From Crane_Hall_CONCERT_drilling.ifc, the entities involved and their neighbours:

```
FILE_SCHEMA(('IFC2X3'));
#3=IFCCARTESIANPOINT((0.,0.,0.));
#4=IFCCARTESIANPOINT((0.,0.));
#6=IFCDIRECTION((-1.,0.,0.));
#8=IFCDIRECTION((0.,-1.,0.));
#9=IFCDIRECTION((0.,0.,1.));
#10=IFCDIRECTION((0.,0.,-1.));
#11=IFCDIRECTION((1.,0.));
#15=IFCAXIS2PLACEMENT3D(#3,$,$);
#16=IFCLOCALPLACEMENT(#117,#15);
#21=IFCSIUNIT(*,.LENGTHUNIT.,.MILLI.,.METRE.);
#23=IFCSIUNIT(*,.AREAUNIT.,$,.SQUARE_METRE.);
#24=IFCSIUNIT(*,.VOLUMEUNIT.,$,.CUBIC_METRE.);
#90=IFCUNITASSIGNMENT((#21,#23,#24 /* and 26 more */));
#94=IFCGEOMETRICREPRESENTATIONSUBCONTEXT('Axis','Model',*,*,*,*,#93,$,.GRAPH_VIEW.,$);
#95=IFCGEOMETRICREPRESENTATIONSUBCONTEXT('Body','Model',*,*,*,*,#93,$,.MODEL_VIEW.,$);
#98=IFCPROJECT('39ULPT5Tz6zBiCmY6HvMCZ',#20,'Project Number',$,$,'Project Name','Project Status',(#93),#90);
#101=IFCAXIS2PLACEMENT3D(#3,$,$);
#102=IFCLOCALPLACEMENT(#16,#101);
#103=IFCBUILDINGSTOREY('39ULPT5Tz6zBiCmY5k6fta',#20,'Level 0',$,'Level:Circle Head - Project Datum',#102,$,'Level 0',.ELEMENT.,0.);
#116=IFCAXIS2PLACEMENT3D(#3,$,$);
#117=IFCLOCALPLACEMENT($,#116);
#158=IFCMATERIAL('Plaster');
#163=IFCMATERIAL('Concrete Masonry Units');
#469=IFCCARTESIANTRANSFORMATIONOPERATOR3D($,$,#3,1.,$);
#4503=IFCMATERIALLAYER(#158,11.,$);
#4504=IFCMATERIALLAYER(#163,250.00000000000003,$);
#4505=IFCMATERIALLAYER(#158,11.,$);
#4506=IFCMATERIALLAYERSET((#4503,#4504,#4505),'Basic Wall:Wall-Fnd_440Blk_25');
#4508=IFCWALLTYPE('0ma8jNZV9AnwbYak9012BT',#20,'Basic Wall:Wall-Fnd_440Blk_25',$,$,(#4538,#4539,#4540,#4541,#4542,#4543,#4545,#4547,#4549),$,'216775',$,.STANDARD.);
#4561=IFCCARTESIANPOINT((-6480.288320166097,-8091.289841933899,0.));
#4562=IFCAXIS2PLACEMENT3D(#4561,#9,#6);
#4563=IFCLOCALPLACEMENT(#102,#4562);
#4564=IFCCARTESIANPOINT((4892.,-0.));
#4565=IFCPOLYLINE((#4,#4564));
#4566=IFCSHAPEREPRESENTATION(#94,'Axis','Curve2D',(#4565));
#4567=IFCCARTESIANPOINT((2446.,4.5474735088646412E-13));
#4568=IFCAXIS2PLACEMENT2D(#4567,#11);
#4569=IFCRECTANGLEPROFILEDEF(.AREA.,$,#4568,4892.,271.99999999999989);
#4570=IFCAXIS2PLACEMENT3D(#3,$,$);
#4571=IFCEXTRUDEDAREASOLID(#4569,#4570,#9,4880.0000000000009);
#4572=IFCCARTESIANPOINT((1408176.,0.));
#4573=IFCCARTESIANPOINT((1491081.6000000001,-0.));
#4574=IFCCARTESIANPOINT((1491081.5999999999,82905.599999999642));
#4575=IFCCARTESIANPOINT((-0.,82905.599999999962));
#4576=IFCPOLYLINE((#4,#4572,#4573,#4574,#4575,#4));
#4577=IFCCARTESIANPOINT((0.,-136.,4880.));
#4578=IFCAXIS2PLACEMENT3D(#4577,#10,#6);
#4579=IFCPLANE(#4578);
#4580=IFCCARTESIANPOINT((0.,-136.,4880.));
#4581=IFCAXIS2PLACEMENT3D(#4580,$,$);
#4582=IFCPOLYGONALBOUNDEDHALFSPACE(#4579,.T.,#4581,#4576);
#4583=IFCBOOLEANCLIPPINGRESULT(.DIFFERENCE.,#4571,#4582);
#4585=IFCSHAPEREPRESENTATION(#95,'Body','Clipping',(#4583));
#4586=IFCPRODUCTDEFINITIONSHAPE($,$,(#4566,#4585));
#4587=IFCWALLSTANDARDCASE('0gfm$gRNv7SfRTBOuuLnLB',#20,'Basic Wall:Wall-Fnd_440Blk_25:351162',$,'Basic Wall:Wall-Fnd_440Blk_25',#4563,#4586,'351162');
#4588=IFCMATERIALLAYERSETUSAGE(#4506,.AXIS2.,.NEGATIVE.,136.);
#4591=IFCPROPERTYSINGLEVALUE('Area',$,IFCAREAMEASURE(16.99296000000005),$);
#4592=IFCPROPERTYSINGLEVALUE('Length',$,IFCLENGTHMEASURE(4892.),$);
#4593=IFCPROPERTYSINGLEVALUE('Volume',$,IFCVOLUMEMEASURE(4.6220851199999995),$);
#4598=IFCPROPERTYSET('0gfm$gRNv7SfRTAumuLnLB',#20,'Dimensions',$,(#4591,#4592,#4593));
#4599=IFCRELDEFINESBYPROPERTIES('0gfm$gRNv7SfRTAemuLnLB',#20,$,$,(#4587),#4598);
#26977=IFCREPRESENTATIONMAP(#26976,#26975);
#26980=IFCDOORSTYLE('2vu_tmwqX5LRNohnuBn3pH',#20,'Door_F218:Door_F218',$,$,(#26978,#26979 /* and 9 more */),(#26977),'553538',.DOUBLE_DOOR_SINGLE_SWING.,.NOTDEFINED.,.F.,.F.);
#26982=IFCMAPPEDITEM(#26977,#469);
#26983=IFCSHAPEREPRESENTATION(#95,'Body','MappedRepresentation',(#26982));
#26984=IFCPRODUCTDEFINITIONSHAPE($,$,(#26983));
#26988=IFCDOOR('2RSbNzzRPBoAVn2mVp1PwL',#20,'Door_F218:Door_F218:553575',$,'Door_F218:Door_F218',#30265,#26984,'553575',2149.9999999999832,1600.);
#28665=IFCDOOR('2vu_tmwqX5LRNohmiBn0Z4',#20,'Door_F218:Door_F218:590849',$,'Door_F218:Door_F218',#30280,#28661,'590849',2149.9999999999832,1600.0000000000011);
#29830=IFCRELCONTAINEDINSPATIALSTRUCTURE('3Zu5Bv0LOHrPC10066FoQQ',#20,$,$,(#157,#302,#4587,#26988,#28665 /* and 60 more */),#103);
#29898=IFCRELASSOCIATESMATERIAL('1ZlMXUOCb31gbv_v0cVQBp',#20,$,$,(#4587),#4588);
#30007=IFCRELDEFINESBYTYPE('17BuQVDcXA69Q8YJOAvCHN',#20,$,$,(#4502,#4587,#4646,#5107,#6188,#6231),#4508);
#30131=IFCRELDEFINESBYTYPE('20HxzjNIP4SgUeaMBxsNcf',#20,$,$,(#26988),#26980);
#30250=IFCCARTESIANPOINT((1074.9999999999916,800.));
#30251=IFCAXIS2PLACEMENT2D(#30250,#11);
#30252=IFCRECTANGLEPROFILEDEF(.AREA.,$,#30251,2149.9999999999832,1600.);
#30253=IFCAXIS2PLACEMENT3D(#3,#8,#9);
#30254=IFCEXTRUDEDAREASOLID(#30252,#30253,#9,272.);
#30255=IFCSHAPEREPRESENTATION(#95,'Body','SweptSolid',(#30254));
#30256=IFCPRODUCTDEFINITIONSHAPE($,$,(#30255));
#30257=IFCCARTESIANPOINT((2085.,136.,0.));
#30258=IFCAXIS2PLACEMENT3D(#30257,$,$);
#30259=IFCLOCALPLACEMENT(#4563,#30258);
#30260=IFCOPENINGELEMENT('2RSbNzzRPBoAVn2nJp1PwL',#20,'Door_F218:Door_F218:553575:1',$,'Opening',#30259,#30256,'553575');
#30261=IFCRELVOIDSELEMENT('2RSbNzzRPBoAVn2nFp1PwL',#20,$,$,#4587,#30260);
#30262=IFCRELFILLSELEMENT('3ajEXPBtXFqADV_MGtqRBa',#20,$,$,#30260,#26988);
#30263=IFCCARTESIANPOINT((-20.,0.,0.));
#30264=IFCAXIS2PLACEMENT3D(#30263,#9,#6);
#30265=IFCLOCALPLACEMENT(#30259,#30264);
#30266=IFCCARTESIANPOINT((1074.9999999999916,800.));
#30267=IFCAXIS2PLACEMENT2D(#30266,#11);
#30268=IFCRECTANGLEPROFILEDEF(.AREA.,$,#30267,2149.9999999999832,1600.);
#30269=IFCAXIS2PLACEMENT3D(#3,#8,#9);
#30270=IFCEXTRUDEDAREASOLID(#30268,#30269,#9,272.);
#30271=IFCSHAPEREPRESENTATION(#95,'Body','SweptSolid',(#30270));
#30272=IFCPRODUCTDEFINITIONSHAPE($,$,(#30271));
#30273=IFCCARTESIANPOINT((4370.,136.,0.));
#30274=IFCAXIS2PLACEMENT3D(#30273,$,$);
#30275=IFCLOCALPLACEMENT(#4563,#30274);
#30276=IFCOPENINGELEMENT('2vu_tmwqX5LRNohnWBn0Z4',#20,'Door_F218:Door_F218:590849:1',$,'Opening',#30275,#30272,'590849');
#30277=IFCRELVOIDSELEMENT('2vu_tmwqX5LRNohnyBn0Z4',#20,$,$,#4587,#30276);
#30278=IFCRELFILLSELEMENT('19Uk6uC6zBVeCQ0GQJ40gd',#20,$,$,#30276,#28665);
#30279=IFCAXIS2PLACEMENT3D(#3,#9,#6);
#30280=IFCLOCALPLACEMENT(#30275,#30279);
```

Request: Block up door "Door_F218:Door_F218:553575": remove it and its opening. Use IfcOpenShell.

```python
import ifcopenshell
import ifcopenshell.api.feature
import ifcopenshell.api.pset
import ifcopenshell.api.root
import ifcopenshell.geom
import ifcopenshell.util.element
import ifcopenshell.util.shape
import ifcopenshell.util.unit

model = ifcopenshell.open("Crane_Hall_CONCERT_drilling.ifc")
area_scale = ifcopenshell.util.unit.calculate_unit_scale(model, "AREAUNIT")
volume_scale = ifcopenshell.util.unit.calculate_unit_scale(model, "VOLUMEUNIT")
settings = ifcopenshell.geom.settings()


def volume(element):
    """Net volume in cubic metres, openings subtracted."""
    shape = ifcopenshell.geom.create_shape(settings, element)
    return ifcopenshell.util.shape.get_volume(shape.geometry)


door = model.by_guid("2RSbNzzRPBoAVn2mVp1PwL")
opening = door.FillsVoids[0].RelatingOpeningElement
wall = opening.VoidsElements[0].RelatingBuildingElement
before = volume(wall)

ifcopenshell.api.root.remove_product(model, product=door)
ifcopenshell.api.feature.remove_feature(model, feature=opening)

after = volume(wall)
thickness = 0.272  # wall thickness in metres

# Update the wall's stored quantities.
pset = model.by_id(ifcopenshell.util.element.get_pset(wall, "Dimensions", should_inherit=False)["id"])
ifcopenshell.api.pset.edit_pset(model, pset=pset, properties={
    "Area": model.create_entity("IfcAreaMeasure", after / thickness / area_scale),
    "Volume": model.create_entity("IfcVolumeMeasure", after / volume_scale),
})

print(f"wall volume {before:.3f} -> {after:.3f} m3")

model.write("Crane_Hall_CONCERT_drilling-out.ifc")
```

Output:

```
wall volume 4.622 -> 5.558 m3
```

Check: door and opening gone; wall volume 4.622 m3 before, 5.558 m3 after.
